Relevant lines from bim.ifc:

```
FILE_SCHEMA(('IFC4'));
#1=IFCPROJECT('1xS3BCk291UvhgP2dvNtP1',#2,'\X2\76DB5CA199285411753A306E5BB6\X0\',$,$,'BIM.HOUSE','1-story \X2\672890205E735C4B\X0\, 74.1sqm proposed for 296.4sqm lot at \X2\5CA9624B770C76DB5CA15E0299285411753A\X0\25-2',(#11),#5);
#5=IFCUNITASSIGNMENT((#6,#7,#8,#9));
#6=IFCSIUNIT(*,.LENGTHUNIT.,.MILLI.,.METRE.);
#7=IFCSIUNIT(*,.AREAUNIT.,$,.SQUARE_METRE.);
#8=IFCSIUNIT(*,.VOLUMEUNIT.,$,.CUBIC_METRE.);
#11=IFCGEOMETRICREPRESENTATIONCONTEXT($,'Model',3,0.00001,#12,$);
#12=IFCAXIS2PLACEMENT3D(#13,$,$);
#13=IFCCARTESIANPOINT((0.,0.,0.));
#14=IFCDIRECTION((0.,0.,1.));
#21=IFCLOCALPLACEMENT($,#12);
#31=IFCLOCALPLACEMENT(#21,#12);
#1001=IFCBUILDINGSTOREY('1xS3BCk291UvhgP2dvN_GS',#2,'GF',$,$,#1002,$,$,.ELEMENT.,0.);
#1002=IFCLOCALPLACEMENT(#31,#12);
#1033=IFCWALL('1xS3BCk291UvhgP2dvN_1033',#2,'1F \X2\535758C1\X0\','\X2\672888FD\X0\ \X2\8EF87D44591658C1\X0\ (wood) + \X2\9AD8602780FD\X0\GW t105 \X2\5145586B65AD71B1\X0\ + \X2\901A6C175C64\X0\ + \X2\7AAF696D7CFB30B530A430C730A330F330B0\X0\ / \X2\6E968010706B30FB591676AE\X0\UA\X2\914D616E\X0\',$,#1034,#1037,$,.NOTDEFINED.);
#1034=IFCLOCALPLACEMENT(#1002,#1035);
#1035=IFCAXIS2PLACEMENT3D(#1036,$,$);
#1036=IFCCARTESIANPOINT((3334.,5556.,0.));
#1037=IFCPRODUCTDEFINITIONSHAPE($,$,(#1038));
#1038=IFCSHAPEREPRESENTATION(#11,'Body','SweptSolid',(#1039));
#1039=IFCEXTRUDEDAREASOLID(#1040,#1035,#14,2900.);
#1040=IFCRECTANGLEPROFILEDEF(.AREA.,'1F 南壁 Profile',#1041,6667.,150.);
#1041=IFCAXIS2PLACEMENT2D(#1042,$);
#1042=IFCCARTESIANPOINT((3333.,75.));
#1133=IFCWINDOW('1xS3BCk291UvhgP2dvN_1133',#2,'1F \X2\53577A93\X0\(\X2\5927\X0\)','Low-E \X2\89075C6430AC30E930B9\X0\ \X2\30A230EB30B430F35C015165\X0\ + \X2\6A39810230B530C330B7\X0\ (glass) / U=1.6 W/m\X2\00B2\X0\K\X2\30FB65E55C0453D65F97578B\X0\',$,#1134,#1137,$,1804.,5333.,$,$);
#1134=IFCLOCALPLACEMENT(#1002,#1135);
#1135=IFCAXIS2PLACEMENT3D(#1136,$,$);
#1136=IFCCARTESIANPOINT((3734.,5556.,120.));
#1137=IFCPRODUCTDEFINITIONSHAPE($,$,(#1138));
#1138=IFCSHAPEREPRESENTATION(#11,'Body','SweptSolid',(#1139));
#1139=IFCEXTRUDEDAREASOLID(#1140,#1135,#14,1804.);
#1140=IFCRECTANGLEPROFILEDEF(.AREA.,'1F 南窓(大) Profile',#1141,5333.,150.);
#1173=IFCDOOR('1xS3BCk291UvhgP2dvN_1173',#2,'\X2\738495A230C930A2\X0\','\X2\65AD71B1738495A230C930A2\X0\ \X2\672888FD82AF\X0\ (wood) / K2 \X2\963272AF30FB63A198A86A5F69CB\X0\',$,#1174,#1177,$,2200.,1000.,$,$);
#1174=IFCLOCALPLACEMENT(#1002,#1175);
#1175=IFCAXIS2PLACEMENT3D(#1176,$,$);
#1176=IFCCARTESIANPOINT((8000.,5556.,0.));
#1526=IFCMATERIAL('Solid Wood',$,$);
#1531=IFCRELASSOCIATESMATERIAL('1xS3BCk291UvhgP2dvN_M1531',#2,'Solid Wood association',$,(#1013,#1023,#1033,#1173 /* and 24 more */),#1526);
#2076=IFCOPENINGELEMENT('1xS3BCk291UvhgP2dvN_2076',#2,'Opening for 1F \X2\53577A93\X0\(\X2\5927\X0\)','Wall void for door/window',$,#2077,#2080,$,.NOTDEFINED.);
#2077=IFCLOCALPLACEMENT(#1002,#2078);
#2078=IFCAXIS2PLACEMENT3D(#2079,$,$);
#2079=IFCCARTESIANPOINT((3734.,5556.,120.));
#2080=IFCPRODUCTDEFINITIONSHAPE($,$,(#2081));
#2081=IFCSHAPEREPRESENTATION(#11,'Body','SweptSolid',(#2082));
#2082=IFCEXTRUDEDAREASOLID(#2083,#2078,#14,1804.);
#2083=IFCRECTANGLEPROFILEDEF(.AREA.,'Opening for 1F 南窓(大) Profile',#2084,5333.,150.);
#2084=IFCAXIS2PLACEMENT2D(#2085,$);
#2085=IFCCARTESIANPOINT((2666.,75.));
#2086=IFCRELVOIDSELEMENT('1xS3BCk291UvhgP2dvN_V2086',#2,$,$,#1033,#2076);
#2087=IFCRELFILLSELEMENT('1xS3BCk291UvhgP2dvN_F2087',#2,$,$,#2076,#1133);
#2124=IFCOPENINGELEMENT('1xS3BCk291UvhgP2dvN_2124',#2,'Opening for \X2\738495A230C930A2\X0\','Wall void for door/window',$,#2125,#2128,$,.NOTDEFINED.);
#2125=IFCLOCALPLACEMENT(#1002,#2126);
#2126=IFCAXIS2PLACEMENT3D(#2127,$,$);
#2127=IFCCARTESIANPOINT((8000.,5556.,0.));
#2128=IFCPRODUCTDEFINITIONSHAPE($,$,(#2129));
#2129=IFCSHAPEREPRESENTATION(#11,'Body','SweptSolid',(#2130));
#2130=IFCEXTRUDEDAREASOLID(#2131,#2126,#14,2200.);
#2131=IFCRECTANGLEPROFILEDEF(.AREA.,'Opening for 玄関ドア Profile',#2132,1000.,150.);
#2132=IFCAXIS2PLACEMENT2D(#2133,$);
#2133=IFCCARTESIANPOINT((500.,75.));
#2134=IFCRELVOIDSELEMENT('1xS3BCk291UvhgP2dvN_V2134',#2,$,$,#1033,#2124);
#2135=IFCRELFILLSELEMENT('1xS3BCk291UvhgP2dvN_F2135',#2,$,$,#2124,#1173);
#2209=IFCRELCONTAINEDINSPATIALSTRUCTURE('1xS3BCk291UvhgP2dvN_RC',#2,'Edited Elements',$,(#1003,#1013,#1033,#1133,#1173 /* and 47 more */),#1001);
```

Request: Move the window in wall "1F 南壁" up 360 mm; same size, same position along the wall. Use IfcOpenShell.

```python
import numpy as np
import ifcopenshell
import ifcopenshell.api.geometry
import ifcopenshell.util.placement
import ifcopenshell.util.unit

model = ifcopenshell.open("bim.ifc")
unit_scale = ifcopenshell.util.unit.calculate_unit_scale(model)

window = model.by_guid("1xS3BCk291UvhgP2dvN_1133")
opening = window.FillsVoids[0].RelatingOpeningElement
dz = 360.0

shift = np.array([0.0, 0.0, dz])
# The window is not placed relative to its opening, so move both.
for product in (opening, window):
    matrix = ifcopenshell.util.placement.get_local_placement(product.ObjectPlacement)
    matrix[:3, 3] += shift
    ifcopenshell.api.geometry.edit_object_placement(model, product=product, matrix=matrix, is_si=False)

print(f"moved by {dz * unit_scale:+.3f} m")

model.write("bim_updated.ifc")
```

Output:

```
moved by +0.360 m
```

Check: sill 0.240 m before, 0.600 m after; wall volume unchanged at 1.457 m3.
